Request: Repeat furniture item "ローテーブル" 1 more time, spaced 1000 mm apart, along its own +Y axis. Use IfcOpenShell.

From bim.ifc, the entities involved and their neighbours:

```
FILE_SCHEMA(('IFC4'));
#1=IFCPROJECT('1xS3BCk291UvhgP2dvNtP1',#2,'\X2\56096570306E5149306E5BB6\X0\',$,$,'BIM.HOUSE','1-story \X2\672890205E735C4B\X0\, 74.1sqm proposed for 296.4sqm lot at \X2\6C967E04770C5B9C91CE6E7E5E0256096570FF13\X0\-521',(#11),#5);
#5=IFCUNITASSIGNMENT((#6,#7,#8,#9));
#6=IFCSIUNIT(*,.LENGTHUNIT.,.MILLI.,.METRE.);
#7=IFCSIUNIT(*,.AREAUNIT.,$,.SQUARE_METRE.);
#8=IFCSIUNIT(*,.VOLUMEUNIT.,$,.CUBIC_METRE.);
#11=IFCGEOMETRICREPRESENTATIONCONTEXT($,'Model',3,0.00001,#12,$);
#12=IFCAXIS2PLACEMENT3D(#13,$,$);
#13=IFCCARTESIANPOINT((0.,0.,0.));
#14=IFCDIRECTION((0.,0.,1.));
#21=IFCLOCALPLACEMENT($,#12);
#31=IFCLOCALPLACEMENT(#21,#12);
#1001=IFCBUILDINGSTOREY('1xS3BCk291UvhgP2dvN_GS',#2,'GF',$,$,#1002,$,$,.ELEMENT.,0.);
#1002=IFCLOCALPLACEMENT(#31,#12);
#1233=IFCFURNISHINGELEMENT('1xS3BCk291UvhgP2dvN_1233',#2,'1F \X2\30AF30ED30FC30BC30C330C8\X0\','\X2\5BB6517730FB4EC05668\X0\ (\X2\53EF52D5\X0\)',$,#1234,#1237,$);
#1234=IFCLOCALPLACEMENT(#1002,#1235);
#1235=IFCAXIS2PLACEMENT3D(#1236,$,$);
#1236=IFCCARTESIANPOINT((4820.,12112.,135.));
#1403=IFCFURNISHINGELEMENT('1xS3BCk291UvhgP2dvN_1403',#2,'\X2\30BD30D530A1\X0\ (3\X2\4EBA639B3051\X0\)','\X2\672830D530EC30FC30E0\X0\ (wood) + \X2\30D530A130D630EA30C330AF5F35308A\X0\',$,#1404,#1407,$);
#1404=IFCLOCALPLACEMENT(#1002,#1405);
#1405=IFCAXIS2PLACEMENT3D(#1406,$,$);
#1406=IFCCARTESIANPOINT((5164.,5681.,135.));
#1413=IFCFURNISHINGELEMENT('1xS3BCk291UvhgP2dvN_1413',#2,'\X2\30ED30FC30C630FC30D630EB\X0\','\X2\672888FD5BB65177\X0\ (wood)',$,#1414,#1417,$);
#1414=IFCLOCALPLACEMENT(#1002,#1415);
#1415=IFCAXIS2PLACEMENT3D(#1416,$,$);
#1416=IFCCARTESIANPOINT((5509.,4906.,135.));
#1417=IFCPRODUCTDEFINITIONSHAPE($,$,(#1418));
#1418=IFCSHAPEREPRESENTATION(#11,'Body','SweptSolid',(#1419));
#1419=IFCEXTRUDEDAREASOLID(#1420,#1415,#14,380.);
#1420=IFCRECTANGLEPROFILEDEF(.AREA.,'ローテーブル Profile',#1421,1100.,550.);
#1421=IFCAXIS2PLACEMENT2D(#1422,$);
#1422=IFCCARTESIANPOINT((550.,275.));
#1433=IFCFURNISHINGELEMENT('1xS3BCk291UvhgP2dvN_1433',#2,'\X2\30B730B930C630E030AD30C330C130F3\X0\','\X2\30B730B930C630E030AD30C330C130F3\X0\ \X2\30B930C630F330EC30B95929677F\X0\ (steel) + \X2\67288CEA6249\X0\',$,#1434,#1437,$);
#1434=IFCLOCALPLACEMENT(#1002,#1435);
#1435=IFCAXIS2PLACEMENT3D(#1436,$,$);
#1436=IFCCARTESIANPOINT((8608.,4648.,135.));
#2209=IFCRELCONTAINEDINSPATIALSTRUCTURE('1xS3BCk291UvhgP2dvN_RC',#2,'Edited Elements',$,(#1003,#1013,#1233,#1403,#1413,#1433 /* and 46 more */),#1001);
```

```python
import ifcopenshell
import ifcopenshell.api.geometry
import ifcopenshell.api.root
import ifcopenshell.util.element
import ifcopenshell.util.placement

model = ifcopenshell.open("bim.ifc")


def reuse_history(source, copy):
    """copy_class also copies each property set's owner history, people and application; keep the originals."""
    for rel in copy.IsDefinedBy:
        if rel.is_a("IfcRelDefinesByProperties") and (history := rel.RelatingPropertyDefinition.OwnerHistory):
            rel.RelatingPropertyDefinition.OwnerHistory = source.OwnerHistory
            ifcopenshell.util.element.remove_deep2(model, history)


source = model.by_guid("1xS3BCk291UvhgP2dvN_1413")
base = ifcopenshell.util.placement.get_local_placement(source.ObjectPlacement)
step = base[:3, 1] * 1000.0

for i in range(1, 2):
    copy = ifcopenshell.api.root.copy_class(model, product=source)
    copy.Representation = ifcopenshell.util.element.copy_deep(
        model, source.Representation, exclude=["IfcGeometricRepresentationContext", "IfcRepresentationMap"]
    )
    reuse_history(source, copy)
    matrix = base.copy()
    matrix[:3, 3] += i * step
    print("added at", matrix[:3, 3].round(3) + 0.0)
    ifcopenshell.api.geometry.edit_object_placement(model, product=copy, matrix=matrix, is_si=False)

model.write("bim_v2.ifc")
```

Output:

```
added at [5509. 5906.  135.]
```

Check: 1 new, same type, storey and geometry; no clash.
